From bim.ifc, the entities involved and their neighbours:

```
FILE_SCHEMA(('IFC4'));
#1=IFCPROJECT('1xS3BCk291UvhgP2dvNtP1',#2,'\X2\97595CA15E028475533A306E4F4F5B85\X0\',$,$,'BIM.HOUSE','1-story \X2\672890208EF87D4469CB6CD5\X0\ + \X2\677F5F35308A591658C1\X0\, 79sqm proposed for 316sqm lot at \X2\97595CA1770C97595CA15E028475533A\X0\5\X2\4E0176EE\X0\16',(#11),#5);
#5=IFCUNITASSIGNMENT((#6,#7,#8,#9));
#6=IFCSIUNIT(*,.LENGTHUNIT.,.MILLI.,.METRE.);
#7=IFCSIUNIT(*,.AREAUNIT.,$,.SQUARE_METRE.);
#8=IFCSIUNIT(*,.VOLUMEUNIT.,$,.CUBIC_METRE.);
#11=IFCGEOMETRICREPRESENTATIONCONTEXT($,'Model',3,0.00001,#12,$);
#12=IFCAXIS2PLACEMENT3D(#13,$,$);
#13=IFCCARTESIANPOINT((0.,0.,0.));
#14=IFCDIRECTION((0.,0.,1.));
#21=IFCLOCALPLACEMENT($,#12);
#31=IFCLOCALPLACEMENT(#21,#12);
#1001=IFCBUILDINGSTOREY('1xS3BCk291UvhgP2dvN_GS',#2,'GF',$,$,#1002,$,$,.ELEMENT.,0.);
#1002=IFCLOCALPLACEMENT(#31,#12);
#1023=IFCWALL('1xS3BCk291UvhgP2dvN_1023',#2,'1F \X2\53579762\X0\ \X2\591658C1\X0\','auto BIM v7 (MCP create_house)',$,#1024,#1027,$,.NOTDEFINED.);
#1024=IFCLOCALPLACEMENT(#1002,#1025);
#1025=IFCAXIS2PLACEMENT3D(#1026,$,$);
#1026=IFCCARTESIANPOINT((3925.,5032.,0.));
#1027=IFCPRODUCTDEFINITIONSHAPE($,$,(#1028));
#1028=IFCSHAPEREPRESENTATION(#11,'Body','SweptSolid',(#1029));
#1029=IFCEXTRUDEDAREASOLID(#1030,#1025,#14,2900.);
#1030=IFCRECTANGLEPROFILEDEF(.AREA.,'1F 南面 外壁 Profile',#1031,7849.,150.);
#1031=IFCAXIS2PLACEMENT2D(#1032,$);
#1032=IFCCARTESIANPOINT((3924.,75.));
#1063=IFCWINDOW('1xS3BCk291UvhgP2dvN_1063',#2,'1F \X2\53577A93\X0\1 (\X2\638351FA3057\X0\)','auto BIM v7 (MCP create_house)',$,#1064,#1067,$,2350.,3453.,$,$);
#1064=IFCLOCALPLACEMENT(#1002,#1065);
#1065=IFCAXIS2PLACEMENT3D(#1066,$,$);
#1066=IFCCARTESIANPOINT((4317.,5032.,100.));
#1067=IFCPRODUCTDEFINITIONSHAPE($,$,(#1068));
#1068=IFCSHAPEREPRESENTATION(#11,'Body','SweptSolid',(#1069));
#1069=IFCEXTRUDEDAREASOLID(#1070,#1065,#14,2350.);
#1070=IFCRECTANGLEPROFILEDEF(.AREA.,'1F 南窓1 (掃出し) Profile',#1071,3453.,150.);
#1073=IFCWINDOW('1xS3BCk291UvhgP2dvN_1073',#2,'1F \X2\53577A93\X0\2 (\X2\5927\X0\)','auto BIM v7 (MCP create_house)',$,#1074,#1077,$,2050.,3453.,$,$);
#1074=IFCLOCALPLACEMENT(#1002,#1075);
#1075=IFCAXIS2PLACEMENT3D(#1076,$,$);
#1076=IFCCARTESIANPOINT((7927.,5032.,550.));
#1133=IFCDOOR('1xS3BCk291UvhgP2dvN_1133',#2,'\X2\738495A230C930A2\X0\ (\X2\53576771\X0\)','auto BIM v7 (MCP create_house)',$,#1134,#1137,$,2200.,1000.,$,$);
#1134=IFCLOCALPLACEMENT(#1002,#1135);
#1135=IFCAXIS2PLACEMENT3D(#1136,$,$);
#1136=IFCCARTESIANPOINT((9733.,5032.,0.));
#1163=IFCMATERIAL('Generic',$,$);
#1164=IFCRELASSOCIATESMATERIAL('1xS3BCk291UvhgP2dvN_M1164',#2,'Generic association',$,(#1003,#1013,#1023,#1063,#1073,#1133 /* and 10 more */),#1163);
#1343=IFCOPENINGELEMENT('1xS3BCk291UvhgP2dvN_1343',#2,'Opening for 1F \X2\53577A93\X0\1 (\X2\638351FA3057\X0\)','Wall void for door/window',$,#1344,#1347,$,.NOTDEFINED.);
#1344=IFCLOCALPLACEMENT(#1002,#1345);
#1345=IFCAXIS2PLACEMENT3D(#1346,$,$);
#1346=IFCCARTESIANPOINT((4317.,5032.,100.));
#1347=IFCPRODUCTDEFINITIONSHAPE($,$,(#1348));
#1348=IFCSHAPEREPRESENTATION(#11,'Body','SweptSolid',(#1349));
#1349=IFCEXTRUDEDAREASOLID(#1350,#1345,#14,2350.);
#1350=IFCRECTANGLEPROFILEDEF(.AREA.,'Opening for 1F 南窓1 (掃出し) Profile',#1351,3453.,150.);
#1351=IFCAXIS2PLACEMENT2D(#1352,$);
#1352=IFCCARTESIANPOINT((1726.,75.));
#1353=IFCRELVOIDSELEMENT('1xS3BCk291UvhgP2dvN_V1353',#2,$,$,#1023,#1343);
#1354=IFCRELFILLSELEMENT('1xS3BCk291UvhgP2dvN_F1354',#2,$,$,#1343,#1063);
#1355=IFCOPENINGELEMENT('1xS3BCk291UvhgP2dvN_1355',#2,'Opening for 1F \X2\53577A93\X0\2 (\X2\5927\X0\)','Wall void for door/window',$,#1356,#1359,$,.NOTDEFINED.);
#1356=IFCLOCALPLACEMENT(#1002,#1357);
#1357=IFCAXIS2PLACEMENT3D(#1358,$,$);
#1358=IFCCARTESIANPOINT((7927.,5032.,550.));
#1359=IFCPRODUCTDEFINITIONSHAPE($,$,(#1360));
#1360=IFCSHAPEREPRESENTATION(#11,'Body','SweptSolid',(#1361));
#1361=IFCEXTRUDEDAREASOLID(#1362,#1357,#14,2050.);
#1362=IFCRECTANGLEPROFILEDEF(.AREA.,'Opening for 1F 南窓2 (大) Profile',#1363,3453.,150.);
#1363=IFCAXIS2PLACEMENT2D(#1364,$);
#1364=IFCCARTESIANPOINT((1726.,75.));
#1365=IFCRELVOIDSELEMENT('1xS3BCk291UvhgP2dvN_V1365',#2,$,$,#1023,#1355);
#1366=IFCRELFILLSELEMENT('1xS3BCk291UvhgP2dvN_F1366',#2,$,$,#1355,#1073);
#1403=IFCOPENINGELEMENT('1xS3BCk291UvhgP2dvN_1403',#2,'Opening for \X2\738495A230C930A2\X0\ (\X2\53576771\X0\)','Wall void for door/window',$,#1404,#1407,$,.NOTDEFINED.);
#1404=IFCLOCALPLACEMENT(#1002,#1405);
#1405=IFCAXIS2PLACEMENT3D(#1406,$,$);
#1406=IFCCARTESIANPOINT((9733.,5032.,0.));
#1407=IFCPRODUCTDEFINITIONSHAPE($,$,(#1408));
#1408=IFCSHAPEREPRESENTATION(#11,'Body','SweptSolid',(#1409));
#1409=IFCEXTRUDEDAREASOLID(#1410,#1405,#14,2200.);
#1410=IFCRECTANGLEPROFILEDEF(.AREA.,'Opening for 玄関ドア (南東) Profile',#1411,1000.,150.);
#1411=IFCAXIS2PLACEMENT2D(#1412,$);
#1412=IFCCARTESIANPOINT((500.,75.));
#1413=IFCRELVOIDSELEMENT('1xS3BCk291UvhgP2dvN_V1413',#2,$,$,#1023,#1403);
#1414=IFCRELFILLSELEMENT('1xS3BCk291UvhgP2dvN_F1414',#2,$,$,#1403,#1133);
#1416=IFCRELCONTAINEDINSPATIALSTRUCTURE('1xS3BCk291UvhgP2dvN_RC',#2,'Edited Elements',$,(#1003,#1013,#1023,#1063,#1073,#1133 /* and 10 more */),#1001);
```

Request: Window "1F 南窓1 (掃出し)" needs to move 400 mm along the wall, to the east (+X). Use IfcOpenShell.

```python
import ifcopenshell
import ifcopenshell.api.geometry
import ifcopenshell.util.placement
import ifcopenshell.util.unit

model = ifcopenshell.open("bim.ifc")
unit_scale = ifcopenshell.util.unit.calculate_unit_scale(model)

window = model.by_guid("1xS3BCk291UvhgP2dvN_1063")
opening = window.FillsVoids[0].RelatingOpeningElement
wall = opening.VoidsElements[0].RelatingBuildingElement

wall_matrix = ifcopenshell.util.placement.get_local_placement(wall.ObjectPlacement)
shift = wall_matrix[:3, 0] * 0.4 / unit_scale
before = ifcopenshell.util.placement.get_local_placement(window.ObjectPlacement)[:3, 3].copy()

# The window is not placed relative to its opening, so move both.
for product in (opening, window):
    matrix = ifcopenshell.util.placement.get_local_placement(product.ObjectPlacement)
    matrix[:3, 3] += shift
    ifcopenshell.api.geometry.edit_object_placement(model, product=product, matrix=matrix, is_si=False)

after = ifcopenshell.util.placement.get_local_placement(window.ObjectPlacement)[:3, 3]
print("window moved by", (after - before).round(3) + 0.0)

model.write("bim_v2.ifc")
```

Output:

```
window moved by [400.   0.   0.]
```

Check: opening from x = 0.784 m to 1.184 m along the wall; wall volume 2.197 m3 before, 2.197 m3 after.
